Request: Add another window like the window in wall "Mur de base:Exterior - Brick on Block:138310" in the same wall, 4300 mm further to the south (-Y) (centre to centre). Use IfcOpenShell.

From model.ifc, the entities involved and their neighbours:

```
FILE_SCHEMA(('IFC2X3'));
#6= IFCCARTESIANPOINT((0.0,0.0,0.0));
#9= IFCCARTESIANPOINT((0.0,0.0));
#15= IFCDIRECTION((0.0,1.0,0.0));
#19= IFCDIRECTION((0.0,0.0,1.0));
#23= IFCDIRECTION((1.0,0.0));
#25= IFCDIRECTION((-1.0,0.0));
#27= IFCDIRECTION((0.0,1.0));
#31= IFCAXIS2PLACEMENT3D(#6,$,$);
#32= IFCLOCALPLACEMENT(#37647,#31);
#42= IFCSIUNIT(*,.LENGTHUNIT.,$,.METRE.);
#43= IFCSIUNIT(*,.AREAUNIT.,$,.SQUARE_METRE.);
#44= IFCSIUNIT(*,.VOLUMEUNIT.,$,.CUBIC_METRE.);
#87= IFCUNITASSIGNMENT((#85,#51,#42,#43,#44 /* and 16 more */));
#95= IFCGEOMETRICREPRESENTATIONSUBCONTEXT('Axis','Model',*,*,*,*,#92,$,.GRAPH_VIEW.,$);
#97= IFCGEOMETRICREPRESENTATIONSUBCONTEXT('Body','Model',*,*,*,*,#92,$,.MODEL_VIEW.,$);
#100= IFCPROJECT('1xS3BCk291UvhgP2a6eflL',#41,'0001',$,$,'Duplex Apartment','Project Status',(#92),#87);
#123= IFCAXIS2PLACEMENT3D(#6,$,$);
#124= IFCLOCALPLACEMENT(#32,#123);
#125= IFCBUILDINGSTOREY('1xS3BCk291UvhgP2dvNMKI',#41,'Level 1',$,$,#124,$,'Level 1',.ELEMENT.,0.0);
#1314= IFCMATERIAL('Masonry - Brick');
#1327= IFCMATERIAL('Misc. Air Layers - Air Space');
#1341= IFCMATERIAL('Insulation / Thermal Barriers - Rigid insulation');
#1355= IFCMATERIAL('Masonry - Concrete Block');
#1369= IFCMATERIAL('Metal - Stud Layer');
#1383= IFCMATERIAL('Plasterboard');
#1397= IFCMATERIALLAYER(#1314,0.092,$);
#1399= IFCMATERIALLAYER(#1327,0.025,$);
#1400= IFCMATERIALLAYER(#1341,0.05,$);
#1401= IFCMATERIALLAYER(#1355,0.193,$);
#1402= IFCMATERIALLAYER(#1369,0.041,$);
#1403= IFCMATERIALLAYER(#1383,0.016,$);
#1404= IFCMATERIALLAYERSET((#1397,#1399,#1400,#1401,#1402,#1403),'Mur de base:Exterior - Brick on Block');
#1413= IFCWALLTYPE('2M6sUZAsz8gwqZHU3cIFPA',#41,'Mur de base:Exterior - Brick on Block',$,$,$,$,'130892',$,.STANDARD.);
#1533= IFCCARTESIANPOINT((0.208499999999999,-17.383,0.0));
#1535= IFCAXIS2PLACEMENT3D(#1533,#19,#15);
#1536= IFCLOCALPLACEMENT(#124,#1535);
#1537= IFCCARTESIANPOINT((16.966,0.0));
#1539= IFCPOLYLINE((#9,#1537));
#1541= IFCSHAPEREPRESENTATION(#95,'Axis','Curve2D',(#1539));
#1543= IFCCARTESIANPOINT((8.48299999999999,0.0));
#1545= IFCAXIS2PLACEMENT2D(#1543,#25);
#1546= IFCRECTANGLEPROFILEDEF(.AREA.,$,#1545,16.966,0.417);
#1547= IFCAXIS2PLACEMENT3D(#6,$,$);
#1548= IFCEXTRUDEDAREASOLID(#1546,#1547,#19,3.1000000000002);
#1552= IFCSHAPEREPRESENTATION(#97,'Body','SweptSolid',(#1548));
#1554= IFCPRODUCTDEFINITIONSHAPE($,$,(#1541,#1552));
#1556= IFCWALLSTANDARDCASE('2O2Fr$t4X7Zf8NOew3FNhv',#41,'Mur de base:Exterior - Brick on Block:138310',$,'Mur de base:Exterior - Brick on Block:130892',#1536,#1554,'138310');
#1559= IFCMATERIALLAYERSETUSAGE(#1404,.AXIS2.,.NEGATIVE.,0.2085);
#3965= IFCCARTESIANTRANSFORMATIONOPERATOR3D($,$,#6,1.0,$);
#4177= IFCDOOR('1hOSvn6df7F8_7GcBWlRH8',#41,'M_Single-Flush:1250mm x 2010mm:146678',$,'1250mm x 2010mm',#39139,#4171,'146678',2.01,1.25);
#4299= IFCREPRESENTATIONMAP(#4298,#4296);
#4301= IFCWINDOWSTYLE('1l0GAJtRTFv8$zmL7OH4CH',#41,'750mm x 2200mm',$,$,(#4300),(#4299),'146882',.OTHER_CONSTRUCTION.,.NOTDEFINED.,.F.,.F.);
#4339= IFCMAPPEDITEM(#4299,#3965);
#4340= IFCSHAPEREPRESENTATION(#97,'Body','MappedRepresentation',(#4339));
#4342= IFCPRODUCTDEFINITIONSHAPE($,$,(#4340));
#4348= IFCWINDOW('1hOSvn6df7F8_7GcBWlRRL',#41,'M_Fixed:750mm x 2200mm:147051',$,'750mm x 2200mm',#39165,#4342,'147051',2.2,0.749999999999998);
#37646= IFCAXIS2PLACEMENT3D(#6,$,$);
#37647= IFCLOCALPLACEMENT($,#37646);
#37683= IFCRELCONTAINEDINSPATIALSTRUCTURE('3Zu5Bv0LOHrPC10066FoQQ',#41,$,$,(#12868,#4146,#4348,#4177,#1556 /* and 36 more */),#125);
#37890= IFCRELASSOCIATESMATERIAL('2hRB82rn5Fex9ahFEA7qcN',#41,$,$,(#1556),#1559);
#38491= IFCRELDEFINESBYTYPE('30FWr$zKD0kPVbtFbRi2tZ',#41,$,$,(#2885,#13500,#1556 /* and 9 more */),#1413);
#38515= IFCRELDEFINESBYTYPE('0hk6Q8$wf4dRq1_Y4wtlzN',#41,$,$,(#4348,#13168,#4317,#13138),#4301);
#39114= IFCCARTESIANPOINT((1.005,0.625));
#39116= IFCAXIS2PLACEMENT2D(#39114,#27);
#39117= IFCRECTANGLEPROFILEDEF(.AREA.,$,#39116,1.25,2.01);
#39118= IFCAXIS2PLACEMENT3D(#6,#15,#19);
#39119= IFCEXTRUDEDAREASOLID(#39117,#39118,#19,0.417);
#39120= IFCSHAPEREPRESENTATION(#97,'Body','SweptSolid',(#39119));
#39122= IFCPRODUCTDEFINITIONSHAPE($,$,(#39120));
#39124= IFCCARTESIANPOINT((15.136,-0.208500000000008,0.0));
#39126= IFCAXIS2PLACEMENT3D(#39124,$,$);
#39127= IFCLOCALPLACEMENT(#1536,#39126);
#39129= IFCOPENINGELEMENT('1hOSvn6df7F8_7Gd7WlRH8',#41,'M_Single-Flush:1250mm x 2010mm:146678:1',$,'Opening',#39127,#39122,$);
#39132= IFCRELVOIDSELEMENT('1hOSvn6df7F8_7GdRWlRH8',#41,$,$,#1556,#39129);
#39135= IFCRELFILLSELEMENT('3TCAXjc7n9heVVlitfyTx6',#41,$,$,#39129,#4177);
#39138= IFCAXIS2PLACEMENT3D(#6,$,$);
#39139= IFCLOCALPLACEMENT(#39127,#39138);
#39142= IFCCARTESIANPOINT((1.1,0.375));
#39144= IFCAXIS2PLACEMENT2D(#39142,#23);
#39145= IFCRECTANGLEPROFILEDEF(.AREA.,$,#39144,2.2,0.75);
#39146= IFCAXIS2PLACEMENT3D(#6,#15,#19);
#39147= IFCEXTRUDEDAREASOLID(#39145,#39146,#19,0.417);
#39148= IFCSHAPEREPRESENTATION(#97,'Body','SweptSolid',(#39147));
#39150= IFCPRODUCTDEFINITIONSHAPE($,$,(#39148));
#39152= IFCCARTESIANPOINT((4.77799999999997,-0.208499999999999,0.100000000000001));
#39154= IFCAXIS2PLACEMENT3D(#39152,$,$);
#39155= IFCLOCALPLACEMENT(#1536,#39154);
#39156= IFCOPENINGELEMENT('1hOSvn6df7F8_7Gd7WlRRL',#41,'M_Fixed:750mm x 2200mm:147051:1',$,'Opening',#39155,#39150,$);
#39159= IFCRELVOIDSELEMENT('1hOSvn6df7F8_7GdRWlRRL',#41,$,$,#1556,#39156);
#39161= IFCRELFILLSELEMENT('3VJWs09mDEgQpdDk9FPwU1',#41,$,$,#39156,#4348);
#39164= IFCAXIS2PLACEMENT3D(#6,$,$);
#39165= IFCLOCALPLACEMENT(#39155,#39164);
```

```python
import ifcopenshell
import ifcopenshell.api.feature
import ifcopenshell.api.geometry
import ifcopenshell.api.root
import ifcopenshell.geom
import ifcopenshell.util.element
import ifcopenshell.util.placement
import ifcopenshell.util.shape
import ifcopenshell.util.unit

model = ifcopenshell.open("model.ifc")
unit_scale = ifcopenshell.util.unit.calculate_unit_scale(model)
settings = ifcopenshell.geom.settings()


def volume(element):
    """Net volume in cubic metres, openings subtracted."""
    shape = ifcopenshell.geom.create_shape(settings, element)
    return ifcopenshell.util.shape.get_volume(shape.geometry)


def reuse_history(source, copy):
    """copy_class also copies each property set's owner history, people and application; keep the originals."""
    for rel in copy.IsDefinedBy:
        if rel.is_a("IfcRelDefinesByProperties") and (history := rel.RelatingPropertyDefinition.OwnerHistory):
            rel.RelatingPropertyDefinition.OwnerHistory = source.OwnerHistory
            ifcopenshell.util.element.remove_deep2(model, history)


window = model.by_guid("1hOSvn6df7F8_7GcBWlRRL")
opening = window.FillsVoids[0].RelatingOpeningElement
wall = opening.VoidsElements[0].RelatingBuildingElement
before = volume(wall)
shift = ifcopenshell.util.placement.get_local_placement(wall.ObjectPlacement)[:3, 0] * -4.3 / unit_scale

# copy_class copies the void relationship, type, container and properties, but no geometry.
new_opening = ifcopenshell.api.root.copy_class(model, product=opening)
new_opening.Representation = ifcopenshell.util.element.copy_deep(
    model, opening.Representation, exclude=["IfcGeometricRepresentationContext", "IfcRepresentationMap"]
)
new_opening.Name = "M_Fixed:750mm x 2200mm"
new_window = ifcopenshell.api.root.copy_class(model, product=window)
new_window.Representation = ifcopenshell.util.element.copy_deep(
    model, window.Representation, exclude=["IfcGeometricRepresentationContext", "IfcRepresentationMap"]
)
new_window.Name = "M_Fixed:750mm x 2200mm"
new_window.Tag = None
reuse_history(window, new_window)
fills = ifcopenshell.api.feature.add_filling(model, opening=new_opening, element=new_window)
fills.OwnerHistory = new_window.OwnerHistory  # required in IFC2X3

for old, new in ((opening, new_opening), (window, new_window)):
    matrix = ifcopenshell.util.placement.get_local_placement(old.ObjectPlacement)
    matrix[:3, 3] += shift
    ifcopenshell.api.geometry.edit_object_placement(model, product=new, matrix=matrix, is_si=False)

after = volume(wall)

print(f"wall volume {before:.3f} -> {after:.3f} m3")

model.write("model_updated.ifc")
```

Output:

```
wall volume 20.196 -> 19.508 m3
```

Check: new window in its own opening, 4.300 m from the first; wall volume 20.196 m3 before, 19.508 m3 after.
